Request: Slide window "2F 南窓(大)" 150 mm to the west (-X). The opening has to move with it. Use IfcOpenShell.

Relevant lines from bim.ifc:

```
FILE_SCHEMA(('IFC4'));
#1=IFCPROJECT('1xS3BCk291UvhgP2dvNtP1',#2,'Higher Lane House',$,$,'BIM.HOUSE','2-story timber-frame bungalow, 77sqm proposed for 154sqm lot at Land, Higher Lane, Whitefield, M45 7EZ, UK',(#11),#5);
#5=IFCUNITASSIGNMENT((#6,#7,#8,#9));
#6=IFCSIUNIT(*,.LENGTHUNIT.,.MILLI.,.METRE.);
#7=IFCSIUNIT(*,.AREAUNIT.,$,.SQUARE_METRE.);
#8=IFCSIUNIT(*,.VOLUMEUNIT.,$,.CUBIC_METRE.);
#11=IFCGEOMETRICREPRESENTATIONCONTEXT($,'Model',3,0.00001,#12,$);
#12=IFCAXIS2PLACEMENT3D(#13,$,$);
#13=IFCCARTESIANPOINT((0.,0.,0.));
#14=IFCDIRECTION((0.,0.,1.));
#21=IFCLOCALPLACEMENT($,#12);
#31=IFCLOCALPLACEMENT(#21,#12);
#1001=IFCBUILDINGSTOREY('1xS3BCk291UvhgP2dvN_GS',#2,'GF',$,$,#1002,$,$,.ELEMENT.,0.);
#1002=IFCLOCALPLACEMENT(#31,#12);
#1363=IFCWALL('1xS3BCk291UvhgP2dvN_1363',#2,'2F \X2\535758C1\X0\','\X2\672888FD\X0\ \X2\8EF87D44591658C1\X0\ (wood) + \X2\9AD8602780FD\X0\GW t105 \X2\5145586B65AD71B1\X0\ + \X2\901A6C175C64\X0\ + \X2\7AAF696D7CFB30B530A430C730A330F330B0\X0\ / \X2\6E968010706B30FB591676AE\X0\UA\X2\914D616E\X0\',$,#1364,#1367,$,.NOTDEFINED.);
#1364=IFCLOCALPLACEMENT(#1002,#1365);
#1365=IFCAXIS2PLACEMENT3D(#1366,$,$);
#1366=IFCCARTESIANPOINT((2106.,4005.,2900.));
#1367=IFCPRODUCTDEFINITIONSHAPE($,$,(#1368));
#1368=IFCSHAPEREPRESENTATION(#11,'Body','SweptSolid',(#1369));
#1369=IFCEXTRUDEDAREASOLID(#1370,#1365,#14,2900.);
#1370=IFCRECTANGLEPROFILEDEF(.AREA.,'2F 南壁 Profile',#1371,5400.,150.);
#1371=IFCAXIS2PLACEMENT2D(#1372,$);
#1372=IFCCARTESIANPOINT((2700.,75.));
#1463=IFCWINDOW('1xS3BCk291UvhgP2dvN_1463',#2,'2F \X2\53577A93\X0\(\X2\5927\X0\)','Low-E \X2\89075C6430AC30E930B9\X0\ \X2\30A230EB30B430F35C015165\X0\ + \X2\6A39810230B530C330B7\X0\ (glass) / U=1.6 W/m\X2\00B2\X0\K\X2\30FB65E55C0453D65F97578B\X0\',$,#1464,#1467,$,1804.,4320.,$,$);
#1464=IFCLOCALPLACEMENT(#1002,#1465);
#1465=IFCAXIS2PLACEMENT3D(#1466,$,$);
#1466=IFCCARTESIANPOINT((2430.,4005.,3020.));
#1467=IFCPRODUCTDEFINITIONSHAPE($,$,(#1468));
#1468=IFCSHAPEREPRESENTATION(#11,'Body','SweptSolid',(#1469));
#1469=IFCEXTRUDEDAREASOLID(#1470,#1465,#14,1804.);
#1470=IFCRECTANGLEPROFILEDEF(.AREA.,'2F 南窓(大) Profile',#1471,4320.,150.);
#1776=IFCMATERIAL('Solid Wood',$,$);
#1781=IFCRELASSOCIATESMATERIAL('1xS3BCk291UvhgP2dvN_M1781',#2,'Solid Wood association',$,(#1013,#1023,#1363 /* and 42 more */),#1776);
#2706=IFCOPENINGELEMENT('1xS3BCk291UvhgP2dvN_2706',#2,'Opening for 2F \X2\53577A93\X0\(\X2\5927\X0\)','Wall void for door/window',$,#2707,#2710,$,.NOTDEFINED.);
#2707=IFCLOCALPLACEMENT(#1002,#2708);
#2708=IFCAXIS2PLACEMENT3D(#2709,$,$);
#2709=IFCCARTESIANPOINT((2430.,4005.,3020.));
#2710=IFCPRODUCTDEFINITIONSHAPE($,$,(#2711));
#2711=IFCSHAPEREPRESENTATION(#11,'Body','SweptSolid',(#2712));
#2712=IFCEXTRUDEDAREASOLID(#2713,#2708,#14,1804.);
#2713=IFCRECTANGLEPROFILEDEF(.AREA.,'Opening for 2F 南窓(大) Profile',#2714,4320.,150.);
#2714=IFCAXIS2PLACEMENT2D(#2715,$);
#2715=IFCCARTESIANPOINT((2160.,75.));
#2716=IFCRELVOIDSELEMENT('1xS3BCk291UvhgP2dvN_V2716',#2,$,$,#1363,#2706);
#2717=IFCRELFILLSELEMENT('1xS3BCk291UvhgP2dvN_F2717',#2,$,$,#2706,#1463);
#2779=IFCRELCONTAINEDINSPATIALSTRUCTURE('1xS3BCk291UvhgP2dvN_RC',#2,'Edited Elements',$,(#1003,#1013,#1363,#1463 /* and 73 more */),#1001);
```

```python
import ifcopenshell
import ifcopenshell.api.geometry
import ifcopenshell.util.placement
import ifcopenshell.util.unit

model = ifcopenshell.open("bim.ifc")
unit_scale = ifcopenshell.util.unit.calculate_unit_scale(model)

window = model.by_guid("1xS3BCk291UvhgP2dvN_1463")
opening = window.FillsVoids[0].RelatingOpeningElement
wall = opening.VoidsElements[0].RelatingBuildingElement

wall_matrix = ifcopenshell.util.placement.get_local_placement(wall.ObjectPlacement)
shift = wall_matrix[:3, 0] * -0.15 / unit_scale
before = ifcopenshell.util.placement.get_local_placement(window.ObjectPlacement)[:3, 3].copy()

# The window is not placed relative to its opening, so move both.
for product in (opening, window):
    matrix = ifcopenshell.util.placement.get_local_placement(product.ObjectPlacement)
    matrix[:3, 3] += shift
    ifcopenshell.api.geometry.edit_object_placement(model, product=product, matrix=matrix, is_si=False)

after = ifcopenshell.util.placement.get_local_placement(window.ObjectPlacement)[:3, 3]
print("window moved by", (after - before).round(3) + 0.0)

model.write("bim_updated.ifc")
```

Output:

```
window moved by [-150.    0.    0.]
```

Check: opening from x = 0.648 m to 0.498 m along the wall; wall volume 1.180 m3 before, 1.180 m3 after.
